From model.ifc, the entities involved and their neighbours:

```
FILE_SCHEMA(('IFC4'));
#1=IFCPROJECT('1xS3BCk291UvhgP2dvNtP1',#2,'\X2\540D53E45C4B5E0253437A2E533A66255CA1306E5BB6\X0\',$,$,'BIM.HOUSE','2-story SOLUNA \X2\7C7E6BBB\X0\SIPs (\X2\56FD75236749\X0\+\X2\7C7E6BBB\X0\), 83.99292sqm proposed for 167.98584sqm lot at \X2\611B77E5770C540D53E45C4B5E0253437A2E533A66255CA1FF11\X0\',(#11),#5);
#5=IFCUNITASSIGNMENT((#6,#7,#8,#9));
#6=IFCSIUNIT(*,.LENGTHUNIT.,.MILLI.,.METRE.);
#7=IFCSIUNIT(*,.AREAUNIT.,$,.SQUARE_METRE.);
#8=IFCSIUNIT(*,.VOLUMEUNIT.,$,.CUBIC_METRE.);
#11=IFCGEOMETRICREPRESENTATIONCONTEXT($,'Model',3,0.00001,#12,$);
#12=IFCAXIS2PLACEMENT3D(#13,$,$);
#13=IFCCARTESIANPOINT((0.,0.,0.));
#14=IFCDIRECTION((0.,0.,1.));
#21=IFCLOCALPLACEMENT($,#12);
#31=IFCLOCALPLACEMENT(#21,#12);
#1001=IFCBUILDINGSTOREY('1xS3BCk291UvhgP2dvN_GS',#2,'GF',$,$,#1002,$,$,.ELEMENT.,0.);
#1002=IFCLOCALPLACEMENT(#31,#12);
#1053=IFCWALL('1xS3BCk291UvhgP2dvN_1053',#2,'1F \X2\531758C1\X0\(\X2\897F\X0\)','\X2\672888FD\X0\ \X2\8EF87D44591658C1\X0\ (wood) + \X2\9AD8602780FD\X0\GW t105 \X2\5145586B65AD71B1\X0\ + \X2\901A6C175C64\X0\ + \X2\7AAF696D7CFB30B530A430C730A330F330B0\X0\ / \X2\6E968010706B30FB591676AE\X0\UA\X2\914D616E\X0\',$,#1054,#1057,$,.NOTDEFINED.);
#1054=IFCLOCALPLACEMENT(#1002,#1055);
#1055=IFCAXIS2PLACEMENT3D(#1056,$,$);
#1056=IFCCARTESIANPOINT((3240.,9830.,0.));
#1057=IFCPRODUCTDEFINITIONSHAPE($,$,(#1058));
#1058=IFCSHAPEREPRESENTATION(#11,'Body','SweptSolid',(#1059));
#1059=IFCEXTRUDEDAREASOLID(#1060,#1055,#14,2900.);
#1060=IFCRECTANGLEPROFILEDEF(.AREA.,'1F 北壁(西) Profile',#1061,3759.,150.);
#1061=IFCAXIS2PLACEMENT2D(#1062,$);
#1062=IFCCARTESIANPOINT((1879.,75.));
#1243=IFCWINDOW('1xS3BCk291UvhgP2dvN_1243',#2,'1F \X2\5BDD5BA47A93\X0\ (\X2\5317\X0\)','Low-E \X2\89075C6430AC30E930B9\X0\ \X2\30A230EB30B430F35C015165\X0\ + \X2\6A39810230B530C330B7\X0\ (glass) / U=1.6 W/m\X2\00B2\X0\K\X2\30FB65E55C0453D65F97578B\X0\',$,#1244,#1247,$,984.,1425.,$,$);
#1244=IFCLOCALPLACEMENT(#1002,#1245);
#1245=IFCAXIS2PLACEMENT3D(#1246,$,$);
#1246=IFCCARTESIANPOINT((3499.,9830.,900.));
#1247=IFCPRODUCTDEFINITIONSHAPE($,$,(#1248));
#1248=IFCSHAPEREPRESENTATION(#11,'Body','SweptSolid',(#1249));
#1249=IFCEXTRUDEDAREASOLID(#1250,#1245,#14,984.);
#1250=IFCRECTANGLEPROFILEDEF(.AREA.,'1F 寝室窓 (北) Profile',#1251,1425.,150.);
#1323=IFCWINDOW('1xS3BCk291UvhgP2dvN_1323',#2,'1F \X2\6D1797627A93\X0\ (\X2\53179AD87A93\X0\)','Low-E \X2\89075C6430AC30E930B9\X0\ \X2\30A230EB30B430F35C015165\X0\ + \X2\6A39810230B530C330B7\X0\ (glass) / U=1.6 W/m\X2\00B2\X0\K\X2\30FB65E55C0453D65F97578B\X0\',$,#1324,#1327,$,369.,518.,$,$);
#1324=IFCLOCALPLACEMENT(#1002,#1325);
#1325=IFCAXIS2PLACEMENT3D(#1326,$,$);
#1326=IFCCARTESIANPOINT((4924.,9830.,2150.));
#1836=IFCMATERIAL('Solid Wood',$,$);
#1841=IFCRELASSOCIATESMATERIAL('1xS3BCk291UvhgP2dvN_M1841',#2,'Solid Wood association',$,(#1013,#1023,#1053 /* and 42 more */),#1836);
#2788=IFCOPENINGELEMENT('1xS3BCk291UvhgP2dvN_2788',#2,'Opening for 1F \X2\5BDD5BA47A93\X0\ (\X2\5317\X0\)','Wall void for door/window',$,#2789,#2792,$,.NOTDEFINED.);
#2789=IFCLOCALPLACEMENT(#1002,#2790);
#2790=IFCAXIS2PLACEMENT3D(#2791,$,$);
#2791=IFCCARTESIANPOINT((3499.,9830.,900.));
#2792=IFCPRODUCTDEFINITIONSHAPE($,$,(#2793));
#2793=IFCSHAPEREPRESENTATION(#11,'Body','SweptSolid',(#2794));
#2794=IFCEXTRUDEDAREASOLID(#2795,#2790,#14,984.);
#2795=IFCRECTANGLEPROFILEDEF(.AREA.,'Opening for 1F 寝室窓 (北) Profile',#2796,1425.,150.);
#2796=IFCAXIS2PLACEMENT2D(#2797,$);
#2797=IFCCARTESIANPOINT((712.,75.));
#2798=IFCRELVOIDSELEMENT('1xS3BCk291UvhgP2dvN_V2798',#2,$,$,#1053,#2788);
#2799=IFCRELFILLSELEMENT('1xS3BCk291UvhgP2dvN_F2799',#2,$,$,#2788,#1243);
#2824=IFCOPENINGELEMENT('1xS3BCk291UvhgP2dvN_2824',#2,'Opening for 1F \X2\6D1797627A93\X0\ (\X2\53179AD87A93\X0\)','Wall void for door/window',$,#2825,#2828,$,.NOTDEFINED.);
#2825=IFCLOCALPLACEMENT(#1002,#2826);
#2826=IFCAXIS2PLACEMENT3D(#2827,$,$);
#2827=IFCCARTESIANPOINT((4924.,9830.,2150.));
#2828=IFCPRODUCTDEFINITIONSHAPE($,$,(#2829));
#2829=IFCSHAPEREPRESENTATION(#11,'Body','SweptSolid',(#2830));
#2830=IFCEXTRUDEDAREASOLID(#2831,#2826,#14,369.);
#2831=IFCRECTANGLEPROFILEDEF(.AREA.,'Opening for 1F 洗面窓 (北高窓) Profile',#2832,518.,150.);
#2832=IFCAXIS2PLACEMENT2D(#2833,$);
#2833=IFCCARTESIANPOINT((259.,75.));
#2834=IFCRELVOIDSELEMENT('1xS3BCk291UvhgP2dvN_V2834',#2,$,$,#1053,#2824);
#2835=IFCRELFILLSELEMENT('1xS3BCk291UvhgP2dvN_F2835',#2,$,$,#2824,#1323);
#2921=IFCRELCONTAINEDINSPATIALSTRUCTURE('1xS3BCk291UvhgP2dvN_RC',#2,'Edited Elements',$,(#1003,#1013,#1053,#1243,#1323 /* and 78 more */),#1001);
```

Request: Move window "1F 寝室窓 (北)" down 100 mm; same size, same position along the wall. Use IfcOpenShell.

```python
import numpy as np
import ifcopenshell
import ifcopenshell.api.geometry
import ifcopenshell.util.placement
import ifcopenshell.util.unit

model = ifcopenshell.open("model.ifc")
unit_scale = ifcopenshell.util.unit.calculate_unit_scale(model)

window = model.by_id(1243)
opening = window.FillsVoids[0].RelatingOpeningElement
dz = -0.1 / unit_scale

shift = np.array([0.0, 0.0, dz])
# The window is not placed relative to its opening, so move both.
for product in (opening, window):
    matrix = ifcopenshell.util.placement.get_local_placement(product.ObjectPlacement)
    matrix[:3, 3] += shift
    ifcopenshell.api.geometry.edit_object_placement(model, product=product, matrix=matrix, is_si=False)

print(f"moved by {dz * unit_scale:+.3f} m")

model.write("model_rev.ifc")
```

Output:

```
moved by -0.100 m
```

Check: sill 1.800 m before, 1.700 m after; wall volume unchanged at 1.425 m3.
